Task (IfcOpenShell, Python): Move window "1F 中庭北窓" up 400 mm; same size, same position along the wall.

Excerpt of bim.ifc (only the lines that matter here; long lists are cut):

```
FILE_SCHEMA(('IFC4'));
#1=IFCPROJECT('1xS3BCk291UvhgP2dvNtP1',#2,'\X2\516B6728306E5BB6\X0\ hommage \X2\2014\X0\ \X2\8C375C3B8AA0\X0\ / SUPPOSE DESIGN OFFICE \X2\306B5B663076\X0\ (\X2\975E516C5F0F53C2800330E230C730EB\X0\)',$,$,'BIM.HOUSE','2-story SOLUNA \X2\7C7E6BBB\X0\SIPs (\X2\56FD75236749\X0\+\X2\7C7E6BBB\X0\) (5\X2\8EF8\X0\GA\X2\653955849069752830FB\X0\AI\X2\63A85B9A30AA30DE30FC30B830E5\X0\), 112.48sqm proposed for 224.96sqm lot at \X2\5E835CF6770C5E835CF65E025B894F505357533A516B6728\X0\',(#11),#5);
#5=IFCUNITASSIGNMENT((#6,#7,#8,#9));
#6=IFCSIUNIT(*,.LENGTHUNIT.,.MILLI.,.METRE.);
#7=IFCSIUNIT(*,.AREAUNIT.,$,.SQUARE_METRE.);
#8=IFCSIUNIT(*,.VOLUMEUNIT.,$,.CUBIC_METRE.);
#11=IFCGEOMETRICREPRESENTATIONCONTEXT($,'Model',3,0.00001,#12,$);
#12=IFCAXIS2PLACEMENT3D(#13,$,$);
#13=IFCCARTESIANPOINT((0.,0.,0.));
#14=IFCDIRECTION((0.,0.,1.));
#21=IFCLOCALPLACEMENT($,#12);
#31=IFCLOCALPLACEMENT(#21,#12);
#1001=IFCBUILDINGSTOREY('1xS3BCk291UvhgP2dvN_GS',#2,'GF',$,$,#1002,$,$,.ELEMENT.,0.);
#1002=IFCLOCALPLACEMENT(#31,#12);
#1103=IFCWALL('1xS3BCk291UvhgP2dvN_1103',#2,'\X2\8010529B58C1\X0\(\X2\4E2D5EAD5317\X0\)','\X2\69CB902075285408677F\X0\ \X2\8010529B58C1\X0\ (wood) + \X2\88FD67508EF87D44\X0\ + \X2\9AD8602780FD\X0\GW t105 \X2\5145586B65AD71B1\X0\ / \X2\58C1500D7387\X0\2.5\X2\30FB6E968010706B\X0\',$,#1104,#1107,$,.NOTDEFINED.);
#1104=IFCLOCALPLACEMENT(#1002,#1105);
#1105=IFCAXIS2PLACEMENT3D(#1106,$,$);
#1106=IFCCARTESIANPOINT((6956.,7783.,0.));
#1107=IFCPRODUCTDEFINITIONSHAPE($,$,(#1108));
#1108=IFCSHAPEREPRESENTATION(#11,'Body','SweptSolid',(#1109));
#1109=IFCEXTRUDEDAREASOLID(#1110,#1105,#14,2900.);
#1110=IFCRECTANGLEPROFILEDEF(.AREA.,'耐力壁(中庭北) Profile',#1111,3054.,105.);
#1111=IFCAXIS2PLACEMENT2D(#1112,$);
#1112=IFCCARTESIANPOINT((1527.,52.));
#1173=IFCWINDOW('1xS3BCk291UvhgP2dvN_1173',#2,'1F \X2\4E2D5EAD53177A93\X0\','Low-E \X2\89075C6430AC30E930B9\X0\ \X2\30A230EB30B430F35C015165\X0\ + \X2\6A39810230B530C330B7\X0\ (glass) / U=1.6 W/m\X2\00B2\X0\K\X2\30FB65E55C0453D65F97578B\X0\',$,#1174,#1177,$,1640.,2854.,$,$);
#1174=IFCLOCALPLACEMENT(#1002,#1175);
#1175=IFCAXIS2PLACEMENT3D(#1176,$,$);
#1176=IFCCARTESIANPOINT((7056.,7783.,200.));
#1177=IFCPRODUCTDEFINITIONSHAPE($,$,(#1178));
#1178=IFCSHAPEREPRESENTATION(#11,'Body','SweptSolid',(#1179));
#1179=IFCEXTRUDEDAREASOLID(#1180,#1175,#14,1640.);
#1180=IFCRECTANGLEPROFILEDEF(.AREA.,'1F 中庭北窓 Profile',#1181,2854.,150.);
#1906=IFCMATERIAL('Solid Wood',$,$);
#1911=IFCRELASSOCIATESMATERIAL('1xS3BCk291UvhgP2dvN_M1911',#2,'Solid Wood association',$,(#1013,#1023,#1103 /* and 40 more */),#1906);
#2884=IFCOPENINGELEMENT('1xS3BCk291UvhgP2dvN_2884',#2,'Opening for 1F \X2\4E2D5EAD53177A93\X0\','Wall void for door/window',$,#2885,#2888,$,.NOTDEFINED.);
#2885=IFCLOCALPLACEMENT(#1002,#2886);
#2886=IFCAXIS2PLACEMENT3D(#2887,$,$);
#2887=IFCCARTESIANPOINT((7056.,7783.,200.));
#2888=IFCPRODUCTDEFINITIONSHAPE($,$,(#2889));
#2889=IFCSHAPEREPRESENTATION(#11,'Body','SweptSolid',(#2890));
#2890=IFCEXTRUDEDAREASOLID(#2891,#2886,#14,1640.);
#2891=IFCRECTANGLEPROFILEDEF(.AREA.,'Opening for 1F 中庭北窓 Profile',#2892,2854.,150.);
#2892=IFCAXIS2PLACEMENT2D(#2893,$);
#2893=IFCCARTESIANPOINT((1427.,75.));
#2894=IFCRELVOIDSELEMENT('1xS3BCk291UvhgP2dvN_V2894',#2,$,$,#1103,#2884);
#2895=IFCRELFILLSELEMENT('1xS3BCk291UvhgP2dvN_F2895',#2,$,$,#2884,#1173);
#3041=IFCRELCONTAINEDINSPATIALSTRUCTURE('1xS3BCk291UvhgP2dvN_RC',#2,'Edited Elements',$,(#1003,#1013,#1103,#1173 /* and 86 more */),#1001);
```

```python
import numpy as np
import ifcopenshell
import ifcopenshell.api.geometry
import ifcopenshell.util.placement
import ifcopenshell.util.unit

model = ifcopenshell.open("bim.ifc")
unit_scale = ifcopenshell.util.unit.calculate_unit_scale(model)

window = model.by_guid("1xS3BCk291UvhgP2dvN_1173")
opening = window.FillsVoids[0].RelatingOpeningElement
dz = 0.4 / unit_scale

shift = np.array([0.0, 0.0, dz])
# The window is not placed relative to its opening, so move both.
for product in (opening, window):
    matrix = ifcopenshell.util.placement.get_local_placement(product.ObjectPlacement)
    matrix[:3, 3] += shift
    ifcopenshell.api.geometry.edit_object_placement(model, product=product, matrix=matrix, is_si=False)

print(f"moved by {dz * unit_scale:+.3f} m")

model.write("bim_edited.ifc")
```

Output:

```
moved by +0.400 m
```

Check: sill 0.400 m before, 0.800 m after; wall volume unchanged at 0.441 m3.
